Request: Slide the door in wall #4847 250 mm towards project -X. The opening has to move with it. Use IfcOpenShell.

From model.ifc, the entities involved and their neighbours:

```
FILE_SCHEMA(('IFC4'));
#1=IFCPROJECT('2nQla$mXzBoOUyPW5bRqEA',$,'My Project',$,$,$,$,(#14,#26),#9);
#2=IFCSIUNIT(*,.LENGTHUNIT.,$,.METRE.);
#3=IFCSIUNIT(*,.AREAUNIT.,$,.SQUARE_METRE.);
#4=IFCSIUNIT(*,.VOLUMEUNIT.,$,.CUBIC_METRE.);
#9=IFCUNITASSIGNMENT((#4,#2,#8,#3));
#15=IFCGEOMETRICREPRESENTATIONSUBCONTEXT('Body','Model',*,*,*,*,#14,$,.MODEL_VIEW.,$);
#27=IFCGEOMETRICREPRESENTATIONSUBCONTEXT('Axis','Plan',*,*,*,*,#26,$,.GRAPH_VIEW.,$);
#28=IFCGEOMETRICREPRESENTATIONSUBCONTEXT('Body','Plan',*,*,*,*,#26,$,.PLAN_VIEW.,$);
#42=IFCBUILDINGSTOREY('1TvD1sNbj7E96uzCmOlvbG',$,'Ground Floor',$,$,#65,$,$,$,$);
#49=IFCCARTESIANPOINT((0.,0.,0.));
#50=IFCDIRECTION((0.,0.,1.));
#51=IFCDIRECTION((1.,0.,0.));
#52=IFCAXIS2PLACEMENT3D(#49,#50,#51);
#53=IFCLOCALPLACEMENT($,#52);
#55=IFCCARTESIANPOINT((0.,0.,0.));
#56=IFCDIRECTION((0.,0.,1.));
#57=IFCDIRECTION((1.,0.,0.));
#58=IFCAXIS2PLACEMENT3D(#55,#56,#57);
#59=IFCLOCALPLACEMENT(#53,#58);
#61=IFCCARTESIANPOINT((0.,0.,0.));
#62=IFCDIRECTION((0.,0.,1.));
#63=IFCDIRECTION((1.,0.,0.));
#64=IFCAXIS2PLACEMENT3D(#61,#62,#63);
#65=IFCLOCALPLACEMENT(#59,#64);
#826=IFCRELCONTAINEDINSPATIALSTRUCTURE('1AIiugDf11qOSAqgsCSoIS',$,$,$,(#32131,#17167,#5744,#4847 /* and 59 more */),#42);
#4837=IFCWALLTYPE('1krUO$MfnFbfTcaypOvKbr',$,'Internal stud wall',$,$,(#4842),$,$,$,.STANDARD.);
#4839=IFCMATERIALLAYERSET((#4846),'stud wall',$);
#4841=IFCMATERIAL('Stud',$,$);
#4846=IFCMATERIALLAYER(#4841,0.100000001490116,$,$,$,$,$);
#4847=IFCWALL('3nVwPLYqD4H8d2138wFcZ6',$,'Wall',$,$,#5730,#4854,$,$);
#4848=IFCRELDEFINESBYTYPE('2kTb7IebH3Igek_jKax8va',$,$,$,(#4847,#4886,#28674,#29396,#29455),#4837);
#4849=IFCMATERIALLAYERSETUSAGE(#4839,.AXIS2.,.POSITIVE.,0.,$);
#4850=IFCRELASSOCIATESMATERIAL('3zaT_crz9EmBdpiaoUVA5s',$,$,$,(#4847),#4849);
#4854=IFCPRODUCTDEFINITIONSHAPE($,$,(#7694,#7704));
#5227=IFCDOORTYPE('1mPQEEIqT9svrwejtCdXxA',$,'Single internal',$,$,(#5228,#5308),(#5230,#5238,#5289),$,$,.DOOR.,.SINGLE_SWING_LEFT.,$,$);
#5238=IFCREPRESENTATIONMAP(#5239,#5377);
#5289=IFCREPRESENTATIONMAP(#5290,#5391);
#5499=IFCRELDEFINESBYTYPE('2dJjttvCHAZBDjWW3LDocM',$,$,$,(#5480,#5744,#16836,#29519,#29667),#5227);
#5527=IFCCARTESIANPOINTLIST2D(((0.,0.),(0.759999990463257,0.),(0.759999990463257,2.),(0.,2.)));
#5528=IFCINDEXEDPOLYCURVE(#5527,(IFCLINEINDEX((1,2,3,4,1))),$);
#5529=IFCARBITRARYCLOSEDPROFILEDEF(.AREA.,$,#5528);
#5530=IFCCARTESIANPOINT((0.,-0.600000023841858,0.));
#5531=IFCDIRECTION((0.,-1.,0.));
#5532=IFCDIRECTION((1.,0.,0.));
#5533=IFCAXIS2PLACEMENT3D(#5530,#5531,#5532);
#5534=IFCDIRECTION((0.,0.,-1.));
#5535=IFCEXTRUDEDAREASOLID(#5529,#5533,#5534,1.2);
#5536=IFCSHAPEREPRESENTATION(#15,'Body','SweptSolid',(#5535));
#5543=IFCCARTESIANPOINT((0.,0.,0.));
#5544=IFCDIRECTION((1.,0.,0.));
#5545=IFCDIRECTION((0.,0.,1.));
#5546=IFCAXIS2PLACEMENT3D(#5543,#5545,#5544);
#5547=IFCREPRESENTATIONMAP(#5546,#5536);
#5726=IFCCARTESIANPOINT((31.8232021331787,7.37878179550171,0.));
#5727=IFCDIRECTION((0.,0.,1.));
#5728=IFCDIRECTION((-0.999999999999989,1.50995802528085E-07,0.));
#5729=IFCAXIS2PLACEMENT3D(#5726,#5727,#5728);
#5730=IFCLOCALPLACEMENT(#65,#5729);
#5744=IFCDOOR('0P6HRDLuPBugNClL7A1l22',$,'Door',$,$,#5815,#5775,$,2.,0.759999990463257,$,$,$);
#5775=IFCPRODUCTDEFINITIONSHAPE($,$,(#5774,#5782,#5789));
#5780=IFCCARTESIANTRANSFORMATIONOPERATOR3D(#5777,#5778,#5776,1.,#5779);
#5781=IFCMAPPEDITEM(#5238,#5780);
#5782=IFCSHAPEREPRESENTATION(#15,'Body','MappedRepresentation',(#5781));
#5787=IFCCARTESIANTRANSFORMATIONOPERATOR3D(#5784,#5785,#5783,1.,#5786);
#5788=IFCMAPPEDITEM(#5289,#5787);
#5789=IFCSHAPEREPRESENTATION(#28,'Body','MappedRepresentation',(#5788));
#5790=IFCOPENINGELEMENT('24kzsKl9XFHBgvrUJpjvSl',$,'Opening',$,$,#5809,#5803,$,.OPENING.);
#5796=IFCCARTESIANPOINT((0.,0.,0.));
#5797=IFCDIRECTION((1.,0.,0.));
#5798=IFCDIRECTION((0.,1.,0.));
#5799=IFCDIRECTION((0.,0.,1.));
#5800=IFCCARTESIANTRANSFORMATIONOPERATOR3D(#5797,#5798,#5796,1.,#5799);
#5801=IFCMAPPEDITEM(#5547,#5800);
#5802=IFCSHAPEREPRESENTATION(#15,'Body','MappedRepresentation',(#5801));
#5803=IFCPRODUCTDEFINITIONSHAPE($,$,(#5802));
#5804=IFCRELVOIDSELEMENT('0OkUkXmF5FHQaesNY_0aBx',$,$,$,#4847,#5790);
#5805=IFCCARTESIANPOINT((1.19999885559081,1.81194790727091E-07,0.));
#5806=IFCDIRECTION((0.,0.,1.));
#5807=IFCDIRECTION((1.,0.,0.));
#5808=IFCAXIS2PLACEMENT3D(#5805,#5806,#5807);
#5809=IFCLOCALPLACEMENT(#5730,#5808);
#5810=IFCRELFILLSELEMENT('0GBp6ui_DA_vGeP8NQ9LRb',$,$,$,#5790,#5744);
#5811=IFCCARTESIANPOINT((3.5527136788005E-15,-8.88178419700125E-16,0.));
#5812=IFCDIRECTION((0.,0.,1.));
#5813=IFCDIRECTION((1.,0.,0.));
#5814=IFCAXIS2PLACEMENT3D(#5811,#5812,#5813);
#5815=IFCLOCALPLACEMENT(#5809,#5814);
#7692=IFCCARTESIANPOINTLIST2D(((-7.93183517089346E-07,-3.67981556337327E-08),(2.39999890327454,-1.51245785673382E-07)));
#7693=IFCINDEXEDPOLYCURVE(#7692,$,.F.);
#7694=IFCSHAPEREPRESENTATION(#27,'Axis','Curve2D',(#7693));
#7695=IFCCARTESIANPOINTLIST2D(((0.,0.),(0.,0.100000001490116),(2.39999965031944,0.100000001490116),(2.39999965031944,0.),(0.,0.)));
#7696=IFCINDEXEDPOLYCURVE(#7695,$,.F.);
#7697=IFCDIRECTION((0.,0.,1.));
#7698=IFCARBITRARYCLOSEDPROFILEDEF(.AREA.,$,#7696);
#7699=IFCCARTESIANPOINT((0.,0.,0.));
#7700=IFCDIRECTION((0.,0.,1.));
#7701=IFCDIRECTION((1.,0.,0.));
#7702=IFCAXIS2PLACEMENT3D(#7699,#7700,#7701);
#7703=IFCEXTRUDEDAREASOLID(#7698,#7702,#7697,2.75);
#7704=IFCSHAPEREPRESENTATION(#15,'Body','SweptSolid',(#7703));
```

```python
import ifcopenshell
import ifcopenshell.api.geometry
import ifcopenshell.util.placement
import ifcopenshell.util.unit

model = ifcopenshell.open("model.ifc")
unit_scale = ifcopenshell.util.unit.calculate_unit_scale(model)

door = model.by_guid("0P6HRDLuPBugNClL7A1l22")
opening = door.FillsVoids[0].RelatingOpeningElement
wall = opening.VoidsElements[0].RelatingBuildingElement

wall_matrix = ifcopenshell.util.placement.get_local_placement(wall.ObjectPlacement)
shift = wall_matrix[:3, 0] * 0.25 / unit_scale
before = ifcopenshell.util.placement.get_local_placement(door.ObjectPlacement)[:3, 3].copy()

# The door is placed relative to its opening, so it follows when the opening moves.
matrix = ifcopenshell.util.placement.get_local_placement(opening.ObjectPlacement)
matrix[:3, 3] += shift
ifcopenshell.api.geometry.edit_object_placement(
    model, product=opening, matrix=matrix, is_si=False, should_transform_children=True
)

after = ifcopenshell.util.placement.get_local_placement(door.ObjectPlacement)[:3, 3]
print("door moved by", (after - before).round(3) + 0.0)

model.write("model_rev.ifc")
```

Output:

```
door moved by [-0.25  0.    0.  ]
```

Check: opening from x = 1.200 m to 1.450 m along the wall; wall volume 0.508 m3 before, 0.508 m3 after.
